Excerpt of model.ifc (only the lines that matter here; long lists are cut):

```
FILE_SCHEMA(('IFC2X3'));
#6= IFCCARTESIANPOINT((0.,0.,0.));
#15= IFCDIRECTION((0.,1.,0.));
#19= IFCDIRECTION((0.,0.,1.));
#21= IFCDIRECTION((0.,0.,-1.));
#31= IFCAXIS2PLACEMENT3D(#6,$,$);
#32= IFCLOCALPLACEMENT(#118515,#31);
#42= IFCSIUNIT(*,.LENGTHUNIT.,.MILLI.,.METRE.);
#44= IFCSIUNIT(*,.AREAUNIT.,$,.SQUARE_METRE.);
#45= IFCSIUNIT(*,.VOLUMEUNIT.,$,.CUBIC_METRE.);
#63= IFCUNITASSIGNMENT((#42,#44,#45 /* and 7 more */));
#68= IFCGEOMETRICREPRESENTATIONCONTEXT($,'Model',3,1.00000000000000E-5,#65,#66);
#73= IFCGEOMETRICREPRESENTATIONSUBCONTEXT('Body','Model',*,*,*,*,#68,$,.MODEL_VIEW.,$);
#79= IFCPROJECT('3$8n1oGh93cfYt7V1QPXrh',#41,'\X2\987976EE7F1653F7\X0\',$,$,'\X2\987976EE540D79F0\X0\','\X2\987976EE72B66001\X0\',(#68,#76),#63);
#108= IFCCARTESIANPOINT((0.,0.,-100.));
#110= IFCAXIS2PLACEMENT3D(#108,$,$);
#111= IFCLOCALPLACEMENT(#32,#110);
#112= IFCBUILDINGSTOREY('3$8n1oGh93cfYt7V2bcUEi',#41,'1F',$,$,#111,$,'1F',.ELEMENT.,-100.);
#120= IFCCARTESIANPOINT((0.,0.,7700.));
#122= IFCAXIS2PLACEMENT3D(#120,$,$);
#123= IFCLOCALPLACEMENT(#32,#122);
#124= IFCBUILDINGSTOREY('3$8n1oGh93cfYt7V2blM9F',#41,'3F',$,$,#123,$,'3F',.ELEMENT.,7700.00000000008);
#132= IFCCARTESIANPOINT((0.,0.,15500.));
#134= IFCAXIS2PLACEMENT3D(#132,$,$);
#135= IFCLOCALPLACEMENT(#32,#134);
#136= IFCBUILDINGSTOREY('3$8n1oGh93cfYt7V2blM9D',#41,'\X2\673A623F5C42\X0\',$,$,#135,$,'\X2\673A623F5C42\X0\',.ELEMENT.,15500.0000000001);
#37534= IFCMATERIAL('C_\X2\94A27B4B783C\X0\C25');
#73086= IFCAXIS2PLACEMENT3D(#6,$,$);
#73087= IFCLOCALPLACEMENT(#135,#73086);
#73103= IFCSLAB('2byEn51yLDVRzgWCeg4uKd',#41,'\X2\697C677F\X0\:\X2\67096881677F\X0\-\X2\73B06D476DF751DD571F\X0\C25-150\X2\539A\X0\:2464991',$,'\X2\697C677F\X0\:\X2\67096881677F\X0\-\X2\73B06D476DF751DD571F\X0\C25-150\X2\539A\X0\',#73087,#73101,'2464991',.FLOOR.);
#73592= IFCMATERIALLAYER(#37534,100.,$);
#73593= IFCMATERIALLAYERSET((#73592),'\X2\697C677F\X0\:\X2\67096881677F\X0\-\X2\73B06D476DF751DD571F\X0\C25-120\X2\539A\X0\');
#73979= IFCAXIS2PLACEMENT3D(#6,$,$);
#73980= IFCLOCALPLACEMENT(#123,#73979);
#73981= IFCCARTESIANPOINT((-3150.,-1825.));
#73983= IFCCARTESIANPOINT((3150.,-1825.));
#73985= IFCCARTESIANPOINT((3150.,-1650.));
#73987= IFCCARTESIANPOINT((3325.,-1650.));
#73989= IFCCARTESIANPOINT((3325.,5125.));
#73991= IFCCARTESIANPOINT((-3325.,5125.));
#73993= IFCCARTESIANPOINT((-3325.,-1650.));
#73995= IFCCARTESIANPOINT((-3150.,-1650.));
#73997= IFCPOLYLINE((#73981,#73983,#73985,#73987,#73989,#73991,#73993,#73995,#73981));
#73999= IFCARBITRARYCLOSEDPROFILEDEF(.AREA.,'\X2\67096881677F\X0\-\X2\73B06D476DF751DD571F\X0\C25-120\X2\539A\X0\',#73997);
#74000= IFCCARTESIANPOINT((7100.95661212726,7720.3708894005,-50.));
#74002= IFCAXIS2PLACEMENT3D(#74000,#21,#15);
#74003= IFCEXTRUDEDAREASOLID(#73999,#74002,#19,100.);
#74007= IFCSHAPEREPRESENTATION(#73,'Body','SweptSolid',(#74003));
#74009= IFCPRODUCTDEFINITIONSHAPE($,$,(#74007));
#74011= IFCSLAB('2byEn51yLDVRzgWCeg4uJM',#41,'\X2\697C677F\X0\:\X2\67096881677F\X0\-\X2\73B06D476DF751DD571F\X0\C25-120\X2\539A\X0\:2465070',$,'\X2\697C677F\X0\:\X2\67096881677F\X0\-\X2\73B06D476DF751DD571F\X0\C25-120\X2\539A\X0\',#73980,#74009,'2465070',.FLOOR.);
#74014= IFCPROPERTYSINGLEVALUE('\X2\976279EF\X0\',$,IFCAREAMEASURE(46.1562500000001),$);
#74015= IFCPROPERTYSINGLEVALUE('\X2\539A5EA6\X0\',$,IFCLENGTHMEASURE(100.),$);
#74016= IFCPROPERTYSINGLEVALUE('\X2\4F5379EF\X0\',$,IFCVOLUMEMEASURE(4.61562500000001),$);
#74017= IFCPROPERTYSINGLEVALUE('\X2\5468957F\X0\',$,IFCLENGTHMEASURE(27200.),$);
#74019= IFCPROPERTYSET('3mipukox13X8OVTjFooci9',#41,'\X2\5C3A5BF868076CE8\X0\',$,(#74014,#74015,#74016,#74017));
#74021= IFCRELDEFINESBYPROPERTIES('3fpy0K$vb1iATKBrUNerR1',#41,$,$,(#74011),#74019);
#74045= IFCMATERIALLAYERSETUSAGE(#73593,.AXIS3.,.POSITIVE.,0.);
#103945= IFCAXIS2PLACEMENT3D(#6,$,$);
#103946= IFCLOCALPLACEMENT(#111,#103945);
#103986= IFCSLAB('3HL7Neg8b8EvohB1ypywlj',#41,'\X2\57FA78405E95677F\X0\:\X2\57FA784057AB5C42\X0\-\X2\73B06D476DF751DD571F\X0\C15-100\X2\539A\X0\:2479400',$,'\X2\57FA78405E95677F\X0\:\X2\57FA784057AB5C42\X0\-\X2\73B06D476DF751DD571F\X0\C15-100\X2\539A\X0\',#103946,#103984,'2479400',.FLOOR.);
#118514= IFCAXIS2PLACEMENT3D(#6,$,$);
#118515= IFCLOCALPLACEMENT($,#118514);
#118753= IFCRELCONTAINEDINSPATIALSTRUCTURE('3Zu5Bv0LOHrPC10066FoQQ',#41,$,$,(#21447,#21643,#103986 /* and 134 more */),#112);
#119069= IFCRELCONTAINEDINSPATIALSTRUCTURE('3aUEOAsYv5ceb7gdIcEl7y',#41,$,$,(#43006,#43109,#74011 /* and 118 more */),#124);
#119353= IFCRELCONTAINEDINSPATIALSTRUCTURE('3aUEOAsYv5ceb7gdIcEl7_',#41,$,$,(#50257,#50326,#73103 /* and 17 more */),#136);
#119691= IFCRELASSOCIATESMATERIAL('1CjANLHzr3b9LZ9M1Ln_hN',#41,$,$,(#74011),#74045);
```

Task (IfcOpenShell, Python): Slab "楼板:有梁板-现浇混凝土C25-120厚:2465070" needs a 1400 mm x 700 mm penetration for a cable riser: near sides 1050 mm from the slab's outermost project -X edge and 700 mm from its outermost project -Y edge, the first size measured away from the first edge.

```python
import numpy as np
import ifcopenshell
import ifcopenshell.api.feature
import ifcopenshell.api.geometry
import ifcopenshell.api.pset
import ifcopenshell.api.root
import ifcopenshell.geom
import ifcopenshell.util.element
import ifcopenshell.util.placement
import ifcopenshell.util.representation
import ifcopenshell.util.shape
import ifcopenshell.util.unit

model = ifcopenshell.open("model.ifc")
unit_scale = ifcopenshell.util.unit.calculate_unit_scale(model)
area_scale = ifcopenshell.util.unit.calculate_unit_scale(model, "AREAUNIT")
volume_scale = ifcopenshell.util.unit.calculate_unit_scale(model, "VOLUMEUNIT")
settings = ifcopenshell.geom.settings()


def volume(element):
    """Net volume in cubic metres, openings subtracted."""
    shape = ifcopenshell.geom.create_shape(settings, element)
    return ifcopenshell.util.shape.get_volume(shape.geometry)


slab = model.by_guid("2byEn51yLDVRzgWCeg4uJM")
before = volume(slab)

# Extent in the slab's own axes, in metres. The edges named are its -X and -Y sides.
slab_shape = ifcopenshell.geom.create_shape(settings, slab)
vertices = ifcopenshell.util.shape.get_vertices(slab_shape.geometry)
x_min, y_min, bottom = vertices.min(axis=0)
top = vertices[:, 2].max()

opening = ifcopenshell.api.root.create_entity(model, ifc_class="IfcOpeningElement", name="Cable riser opening")
context = ifcopenshell.util.representation.get_context(model, "Model", "Body", "MODEL_VIEW")
width, depth = 1.4, 0.7
outline = [(0.0, 0.0), (width, 0.0), (width, depth), (0.0, depth), (0.0, 0.0)]
# Overshoot both faces by 50 mm so the cut is clean.
shape = ifcopenshell.api.geometry.add_slab_representation(
    model, context=context, depth=top - bottom + 0.1, polyline=outline
)
ifcopenshell.api.geometry.assign_representation(model, product=opening, representation=shape)

matrix = ifcopenshell.util.placement.get_local_placement(slab.ObjectPlacement)
matrix[:, 3] = matrix @ np.append(np.array([x_min + 1.05, y_min + 0.7, bottom - 0.05]) / unit_scale, 1.0)
ifcopenshell.api.geometry.edit_object_placement(model, product=opening, matrix=matrix, is_si=False)
ifcopenshell.api.feature.add_feature(model, feature=opening, element=slab)

after = volume(slab)

# Update the slab's stored quantities.
pset = model.by_id(ifcopenshell.util.element.get_pset(slab, "尺寸标注", should_inherit=False)["id"])
ifcopenshell.api.pset.edit_pset(model, pset=pset, properties={
    "面积": model.create_entity("IfcAreaMeasure", after / (top - bottom) / area_scale),
    "体积": model.create_entity("IfcVolumeMeasure", after / volume_scale),
})

print(f"slab volume {before:.3f} -> {after:.3f} m3")

model.write("model-out.ifc")
```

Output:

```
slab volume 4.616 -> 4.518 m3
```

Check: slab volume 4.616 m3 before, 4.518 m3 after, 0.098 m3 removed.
